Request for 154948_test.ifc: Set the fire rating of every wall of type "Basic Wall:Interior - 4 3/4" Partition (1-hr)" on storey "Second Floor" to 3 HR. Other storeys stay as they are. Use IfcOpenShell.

First a look at what the model holds.

```python
import ifcopenshell
import ifcopenshell.util.element

model = ifcopenshell.open("154948_test.ifc")
print(model.schema)
storey = next(s for s in model.by_type("IfcBuildingStorey") if s.Name == "Second Floor")
walls = [e for e in ifcopenshell.util.element.get_decomposition(storey) if e.is_a("IfcWall")]
seen = {}
for e in walls:
    element_type = ifcopenshell.util.element.get_type(e)
    key = (element_type.Name if element_type != e and element_type else None, ifcopenshell.util.element.get_pset(e, "Pset_WallCommon", "FireRating"))
    seen[key] = seen.get(key, 0) + 1
for (name, value), count in sorted(seen.items(), key=str):
    print(count, "x", name, "|", value)
```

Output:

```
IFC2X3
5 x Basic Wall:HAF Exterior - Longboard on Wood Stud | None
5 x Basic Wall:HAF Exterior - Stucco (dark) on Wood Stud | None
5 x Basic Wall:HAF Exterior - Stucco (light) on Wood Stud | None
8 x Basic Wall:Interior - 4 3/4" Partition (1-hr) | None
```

```python
import ifcopenshell
import ifcopenshell.api.pset
import ifcopenshell.util.element

model = ifcopenshell.open("154948_test.ifc")

storey = next(s for s in model.by_type("IfcBuildingStorey") if s.Name == "Second Floor")
walls = [e for e in ifcopenshell.util.element.get_decomposition(storey) if e.is_a("IfcWall")]

count = 0
for e in walls:
    element_type = ifcopenshell.util.element.get_type(e)
    if element_type in (None, e) or element_type.Name != 'Basic Wall:Interior - 4 3/4" Partition (1-hr)':
        continue
    # add_pset returns the element's existing set when there is one.
    pset = ifcopenshell.api.pset.add_pset(model, product=e, name="Pset_WallCommon")
    ifcopenshell.api.pset.edit_pset(model, pset=pset, properties={"FireRating": "3 HR"})
    count += 1

print(count, "walls updated")

model.write("154948_test_edited.ifc")
```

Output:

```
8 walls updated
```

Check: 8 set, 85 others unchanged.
